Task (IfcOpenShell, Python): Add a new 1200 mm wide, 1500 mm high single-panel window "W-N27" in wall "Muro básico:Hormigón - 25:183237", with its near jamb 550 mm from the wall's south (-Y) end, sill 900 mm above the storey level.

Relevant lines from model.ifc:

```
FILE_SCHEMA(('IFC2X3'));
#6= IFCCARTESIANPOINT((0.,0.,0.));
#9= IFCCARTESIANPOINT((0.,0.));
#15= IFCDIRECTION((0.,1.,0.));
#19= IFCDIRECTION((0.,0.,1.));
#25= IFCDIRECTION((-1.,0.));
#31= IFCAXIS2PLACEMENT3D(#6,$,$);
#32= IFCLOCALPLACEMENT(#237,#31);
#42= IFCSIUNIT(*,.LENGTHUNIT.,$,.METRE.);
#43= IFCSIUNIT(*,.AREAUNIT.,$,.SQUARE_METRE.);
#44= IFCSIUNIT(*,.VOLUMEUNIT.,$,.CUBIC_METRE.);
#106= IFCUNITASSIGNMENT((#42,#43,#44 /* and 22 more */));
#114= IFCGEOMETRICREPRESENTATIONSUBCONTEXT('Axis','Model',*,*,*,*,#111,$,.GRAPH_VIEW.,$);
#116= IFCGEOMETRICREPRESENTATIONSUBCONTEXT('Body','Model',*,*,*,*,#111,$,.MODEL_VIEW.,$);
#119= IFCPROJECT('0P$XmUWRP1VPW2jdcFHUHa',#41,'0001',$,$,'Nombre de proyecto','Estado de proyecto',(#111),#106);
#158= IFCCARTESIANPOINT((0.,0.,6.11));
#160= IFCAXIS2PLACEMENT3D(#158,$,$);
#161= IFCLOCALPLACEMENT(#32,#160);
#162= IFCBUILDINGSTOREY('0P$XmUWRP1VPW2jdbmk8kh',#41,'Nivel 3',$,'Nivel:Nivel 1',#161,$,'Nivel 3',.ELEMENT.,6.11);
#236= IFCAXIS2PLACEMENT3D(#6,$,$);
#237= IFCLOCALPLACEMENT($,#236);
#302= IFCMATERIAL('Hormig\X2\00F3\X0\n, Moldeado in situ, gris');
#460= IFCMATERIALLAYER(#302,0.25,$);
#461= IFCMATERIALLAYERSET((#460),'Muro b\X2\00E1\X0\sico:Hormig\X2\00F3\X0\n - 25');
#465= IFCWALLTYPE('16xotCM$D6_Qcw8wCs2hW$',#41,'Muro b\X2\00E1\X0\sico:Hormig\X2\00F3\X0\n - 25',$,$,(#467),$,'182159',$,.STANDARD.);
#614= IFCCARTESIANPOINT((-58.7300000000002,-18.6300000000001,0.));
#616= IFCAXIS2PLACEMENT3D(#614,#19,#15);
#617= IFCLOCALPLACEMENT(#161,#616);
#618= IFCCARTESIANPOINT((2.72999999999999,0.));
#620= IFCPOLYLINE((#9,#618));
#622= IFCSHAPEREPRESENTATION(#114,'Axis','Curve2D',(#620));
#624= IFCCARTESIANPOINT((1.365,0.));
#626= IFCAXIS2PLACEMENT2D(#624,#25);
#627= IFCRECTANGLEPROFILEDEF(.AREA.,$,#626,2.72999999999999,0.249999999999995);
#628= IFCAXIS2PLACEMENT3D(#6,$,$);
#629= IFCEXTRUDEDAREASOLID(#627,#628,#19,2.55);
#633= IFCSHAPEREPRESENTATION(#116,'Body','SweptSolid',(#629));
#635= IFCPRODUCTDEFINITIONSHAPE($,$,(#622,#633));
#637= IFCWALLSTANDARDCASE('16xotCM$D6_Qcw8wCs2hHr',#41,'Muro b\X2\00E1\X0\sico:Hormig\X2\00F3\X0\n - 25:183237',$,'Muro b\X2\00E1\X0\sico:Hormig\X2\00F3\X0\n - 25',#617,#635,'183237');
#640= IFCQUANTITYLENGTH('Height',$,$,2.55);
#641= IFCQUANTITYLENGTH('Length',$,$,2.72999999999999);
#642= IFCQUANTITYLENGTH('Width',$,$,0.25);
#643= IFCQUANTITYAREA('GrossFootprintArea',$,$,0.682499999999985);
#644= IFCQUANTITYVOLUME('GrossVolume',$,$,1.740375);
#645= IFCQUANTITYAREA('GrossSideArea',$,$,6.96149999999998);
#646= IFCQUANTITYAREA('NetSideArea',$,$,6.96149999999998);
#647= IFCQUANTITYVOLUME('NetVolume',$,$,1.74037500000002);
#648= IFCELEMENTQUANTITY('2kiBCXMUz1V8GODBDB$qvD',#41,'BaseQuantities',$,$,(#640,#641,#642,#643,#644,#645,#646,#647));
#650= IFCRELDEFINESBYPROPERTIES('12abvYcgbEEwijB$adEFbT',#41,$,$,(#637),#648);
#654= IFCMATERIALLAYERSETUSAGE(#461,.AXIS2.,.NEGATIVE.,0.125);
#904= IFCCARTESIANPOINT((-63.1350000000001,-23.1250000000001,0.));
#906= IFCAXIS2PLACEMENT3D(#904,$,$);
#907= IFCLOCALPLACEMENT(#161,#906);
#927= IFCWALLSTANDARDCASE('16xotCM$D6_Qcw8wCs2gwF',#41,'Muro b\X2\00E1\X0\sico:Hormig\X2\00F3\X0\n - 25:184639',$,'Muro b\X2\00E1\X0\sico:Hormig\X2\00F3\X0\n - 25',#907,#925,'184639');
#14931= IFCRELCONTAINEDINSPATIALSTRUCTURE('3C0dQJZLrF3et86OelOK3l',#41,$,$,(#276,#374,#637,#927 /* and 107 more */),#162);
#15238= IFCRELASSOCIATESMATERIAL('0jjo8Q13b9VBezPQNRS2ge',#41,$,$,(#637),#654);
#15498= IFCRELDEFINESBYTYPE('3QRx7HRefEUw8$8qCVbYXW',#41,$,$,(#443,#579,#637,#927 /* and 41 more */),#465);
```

```python
import numpy as np
import ifcopenshell
import ifcopenshell.api.feature
import ifcopenshell.api.geometry
import ifcopenshell.api.pset
import ifcopenshell.api.root
import ifcopenshell.api.spatial
import ifcopenshell.api.type
import ifcopenshell.geom
import ifcopenshell.util.element
import ifcopenshell.util.placement
import ifcopenshell.util.representation
import ifcopenshell.util.shape
import ifcopenshell.util.unit

model = ifcopenshell.open("model.ifc")
unit_scale = ifcopenshell.util.unit.calculate_unit_scale(model)
area_scale = ifcopenshell.util.unit.calculate_unit_scale(model, "AREAUNIT")
volume_scale = ifcopenshell.util.unit.calculate_unit_scale(model, "VOLUMEUNIT")
settings = ifcopenshell.geom.settings()


def volume(element):
    """Net volume in cubic metres, openings subtracted."""
    shape = ifcopenshell.geom.create_shape(settings, element)
    return ifcopenshell.util.shape.get_volume(shape.geometry)


wall = model.by_guid("16xotCM$D6_Qcw8wCs2hHr")
storey = ifcopenshell.util.element.get_container(wall, ifc_class="IfcBuildingStorey")
context = ifcopenshell.util.representation.get_context(model, "Model", "Body", "MODEL_VIEW")
before = volume(wall)

width, height, from_end, sill = 1.2, 1.5, 0.55, 0.9  # metres

# The wall runs along its own X axis, and the end named is its -X end.
wall_shape = ifcopenshell.geom.create_shape(settings, wall)
x, y, z = ifcopenshell.util.shape.get_vertices(wall_shape.geometry).T
start = x.min() + from_end
face, thickness = float(y.min()), float(y.max() - y.min())
wall_matrix = ifcopenshell.util.placement.get_local_placement(wall.ObjectPlacement)
level = ifcopenshell.util.placement.get_local_placement(storey.ObjectPlacement)[2, 3]


def in_wall(x, y):
    """Placement at x, y metres in the wall's axes, at sill height."""
    matrix = wall_matrix.copy()
    matrix[:, 3] = wall_matrix @ np.array([x / unit_scale, y / unit_scale, 0.0, 1.0])
    matrix[2, 3] = level + sill / unit_scale
    return matrix


# Opening: a box that overshoots both wall faces by 50 mm.
opening = ifcopenshell.api.root.create_entity(model, ifc_class="IfcOpeningElement")
box = ifcopenshell.api.geometry.add_wall_representation(
    model, context=context, length=width, height=height, thickness=thickness + 0.1
)
ifcopenshell.api.geometry.assign_representation(model, product=opening, representation=box)
ifcopenshell.api.geometry.edit_object_placement(model, product=opening, matrix=in_wall(start, face - 0.05), is_si=False)
ifcopenshell.api.feature.add_feature(model, feature=opening, element=wall)

window = ifcopenshell.api.root.create_entity(model, ifc_class="IfcWindow", name="W-N27")
window.OverallWidth, window.OverallHeight = width / unit_scale, height / unit_scale
body = ifcopenshell.api.geometry.add_window_representation(
    model,
    context=context,
    overall_width=window.OverallWidth,
    overall_height=window.OverallHeight,
    partition_type="SINGLE_PANEL",
)
ifcopenshell.api.geometry.assign_representation(model, product=window, representation=body)
ifcopenshell.api.spatial.assign_container(model, products=[window], relating_structure=storey)
fills = ifcopenshell.api.feature.add_filling(model, opening=opening, element=window)
fills.OwnerHistory = window.OwnerHistory  # required in IFC2X3

# IFC2X3 keeps the operation on the window style.
style = ifcopenshell.api.root.create_entity(model, ifc_class="IfcWindowStyle", name="W-N27")
style.OperationType, style.ConstructionType = "SINGLE_PANEL", "NOTDEFINED"
style.ParameterTakesPrecedence = style.Sizeable = False
ifcopenshell.api.type.assign_type(model, related_objects=[window], relating_type=style)

# Centre the window in the wall's thickness.
ifcopenshell.api.geometry.edit_object_placement(model, product=window, matrix=in_wall(start, face), is_si=False)
window_shape = ifcopenshell.geom.create_shape(settings, window)
depth = ifcopenshell.util.shape.get_vertices(window_shape.geometry)[:, 1]
offset = face + thickness / 2 - (depth.min() + depth.max()) / 2
ifcopenshell.api.geometry.edit_object_placement(model, product=window, matrix=in_wall(start, offset), is_si=False)

after = volume(wall)

# Update the wall's stored quantities.
qto = model.by_id(ifcopenshell.util.element.get_pset(wall, "BaseQuantities", should_inherit=False)["id"])
ifcopenshell.api.pset.edit_qto(model, qto=qto, properties={
    "NetSideArea": after / thickness / area_scale,
    "NetVolume": after / volume_scale,
})

print(f"wall volume {before:.3f} -> {after:.3f} m3")

model.write("model_rev.ifc")
```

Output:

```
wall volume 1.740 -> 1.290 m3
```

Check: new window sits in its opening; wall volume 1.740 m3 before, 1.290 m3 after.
